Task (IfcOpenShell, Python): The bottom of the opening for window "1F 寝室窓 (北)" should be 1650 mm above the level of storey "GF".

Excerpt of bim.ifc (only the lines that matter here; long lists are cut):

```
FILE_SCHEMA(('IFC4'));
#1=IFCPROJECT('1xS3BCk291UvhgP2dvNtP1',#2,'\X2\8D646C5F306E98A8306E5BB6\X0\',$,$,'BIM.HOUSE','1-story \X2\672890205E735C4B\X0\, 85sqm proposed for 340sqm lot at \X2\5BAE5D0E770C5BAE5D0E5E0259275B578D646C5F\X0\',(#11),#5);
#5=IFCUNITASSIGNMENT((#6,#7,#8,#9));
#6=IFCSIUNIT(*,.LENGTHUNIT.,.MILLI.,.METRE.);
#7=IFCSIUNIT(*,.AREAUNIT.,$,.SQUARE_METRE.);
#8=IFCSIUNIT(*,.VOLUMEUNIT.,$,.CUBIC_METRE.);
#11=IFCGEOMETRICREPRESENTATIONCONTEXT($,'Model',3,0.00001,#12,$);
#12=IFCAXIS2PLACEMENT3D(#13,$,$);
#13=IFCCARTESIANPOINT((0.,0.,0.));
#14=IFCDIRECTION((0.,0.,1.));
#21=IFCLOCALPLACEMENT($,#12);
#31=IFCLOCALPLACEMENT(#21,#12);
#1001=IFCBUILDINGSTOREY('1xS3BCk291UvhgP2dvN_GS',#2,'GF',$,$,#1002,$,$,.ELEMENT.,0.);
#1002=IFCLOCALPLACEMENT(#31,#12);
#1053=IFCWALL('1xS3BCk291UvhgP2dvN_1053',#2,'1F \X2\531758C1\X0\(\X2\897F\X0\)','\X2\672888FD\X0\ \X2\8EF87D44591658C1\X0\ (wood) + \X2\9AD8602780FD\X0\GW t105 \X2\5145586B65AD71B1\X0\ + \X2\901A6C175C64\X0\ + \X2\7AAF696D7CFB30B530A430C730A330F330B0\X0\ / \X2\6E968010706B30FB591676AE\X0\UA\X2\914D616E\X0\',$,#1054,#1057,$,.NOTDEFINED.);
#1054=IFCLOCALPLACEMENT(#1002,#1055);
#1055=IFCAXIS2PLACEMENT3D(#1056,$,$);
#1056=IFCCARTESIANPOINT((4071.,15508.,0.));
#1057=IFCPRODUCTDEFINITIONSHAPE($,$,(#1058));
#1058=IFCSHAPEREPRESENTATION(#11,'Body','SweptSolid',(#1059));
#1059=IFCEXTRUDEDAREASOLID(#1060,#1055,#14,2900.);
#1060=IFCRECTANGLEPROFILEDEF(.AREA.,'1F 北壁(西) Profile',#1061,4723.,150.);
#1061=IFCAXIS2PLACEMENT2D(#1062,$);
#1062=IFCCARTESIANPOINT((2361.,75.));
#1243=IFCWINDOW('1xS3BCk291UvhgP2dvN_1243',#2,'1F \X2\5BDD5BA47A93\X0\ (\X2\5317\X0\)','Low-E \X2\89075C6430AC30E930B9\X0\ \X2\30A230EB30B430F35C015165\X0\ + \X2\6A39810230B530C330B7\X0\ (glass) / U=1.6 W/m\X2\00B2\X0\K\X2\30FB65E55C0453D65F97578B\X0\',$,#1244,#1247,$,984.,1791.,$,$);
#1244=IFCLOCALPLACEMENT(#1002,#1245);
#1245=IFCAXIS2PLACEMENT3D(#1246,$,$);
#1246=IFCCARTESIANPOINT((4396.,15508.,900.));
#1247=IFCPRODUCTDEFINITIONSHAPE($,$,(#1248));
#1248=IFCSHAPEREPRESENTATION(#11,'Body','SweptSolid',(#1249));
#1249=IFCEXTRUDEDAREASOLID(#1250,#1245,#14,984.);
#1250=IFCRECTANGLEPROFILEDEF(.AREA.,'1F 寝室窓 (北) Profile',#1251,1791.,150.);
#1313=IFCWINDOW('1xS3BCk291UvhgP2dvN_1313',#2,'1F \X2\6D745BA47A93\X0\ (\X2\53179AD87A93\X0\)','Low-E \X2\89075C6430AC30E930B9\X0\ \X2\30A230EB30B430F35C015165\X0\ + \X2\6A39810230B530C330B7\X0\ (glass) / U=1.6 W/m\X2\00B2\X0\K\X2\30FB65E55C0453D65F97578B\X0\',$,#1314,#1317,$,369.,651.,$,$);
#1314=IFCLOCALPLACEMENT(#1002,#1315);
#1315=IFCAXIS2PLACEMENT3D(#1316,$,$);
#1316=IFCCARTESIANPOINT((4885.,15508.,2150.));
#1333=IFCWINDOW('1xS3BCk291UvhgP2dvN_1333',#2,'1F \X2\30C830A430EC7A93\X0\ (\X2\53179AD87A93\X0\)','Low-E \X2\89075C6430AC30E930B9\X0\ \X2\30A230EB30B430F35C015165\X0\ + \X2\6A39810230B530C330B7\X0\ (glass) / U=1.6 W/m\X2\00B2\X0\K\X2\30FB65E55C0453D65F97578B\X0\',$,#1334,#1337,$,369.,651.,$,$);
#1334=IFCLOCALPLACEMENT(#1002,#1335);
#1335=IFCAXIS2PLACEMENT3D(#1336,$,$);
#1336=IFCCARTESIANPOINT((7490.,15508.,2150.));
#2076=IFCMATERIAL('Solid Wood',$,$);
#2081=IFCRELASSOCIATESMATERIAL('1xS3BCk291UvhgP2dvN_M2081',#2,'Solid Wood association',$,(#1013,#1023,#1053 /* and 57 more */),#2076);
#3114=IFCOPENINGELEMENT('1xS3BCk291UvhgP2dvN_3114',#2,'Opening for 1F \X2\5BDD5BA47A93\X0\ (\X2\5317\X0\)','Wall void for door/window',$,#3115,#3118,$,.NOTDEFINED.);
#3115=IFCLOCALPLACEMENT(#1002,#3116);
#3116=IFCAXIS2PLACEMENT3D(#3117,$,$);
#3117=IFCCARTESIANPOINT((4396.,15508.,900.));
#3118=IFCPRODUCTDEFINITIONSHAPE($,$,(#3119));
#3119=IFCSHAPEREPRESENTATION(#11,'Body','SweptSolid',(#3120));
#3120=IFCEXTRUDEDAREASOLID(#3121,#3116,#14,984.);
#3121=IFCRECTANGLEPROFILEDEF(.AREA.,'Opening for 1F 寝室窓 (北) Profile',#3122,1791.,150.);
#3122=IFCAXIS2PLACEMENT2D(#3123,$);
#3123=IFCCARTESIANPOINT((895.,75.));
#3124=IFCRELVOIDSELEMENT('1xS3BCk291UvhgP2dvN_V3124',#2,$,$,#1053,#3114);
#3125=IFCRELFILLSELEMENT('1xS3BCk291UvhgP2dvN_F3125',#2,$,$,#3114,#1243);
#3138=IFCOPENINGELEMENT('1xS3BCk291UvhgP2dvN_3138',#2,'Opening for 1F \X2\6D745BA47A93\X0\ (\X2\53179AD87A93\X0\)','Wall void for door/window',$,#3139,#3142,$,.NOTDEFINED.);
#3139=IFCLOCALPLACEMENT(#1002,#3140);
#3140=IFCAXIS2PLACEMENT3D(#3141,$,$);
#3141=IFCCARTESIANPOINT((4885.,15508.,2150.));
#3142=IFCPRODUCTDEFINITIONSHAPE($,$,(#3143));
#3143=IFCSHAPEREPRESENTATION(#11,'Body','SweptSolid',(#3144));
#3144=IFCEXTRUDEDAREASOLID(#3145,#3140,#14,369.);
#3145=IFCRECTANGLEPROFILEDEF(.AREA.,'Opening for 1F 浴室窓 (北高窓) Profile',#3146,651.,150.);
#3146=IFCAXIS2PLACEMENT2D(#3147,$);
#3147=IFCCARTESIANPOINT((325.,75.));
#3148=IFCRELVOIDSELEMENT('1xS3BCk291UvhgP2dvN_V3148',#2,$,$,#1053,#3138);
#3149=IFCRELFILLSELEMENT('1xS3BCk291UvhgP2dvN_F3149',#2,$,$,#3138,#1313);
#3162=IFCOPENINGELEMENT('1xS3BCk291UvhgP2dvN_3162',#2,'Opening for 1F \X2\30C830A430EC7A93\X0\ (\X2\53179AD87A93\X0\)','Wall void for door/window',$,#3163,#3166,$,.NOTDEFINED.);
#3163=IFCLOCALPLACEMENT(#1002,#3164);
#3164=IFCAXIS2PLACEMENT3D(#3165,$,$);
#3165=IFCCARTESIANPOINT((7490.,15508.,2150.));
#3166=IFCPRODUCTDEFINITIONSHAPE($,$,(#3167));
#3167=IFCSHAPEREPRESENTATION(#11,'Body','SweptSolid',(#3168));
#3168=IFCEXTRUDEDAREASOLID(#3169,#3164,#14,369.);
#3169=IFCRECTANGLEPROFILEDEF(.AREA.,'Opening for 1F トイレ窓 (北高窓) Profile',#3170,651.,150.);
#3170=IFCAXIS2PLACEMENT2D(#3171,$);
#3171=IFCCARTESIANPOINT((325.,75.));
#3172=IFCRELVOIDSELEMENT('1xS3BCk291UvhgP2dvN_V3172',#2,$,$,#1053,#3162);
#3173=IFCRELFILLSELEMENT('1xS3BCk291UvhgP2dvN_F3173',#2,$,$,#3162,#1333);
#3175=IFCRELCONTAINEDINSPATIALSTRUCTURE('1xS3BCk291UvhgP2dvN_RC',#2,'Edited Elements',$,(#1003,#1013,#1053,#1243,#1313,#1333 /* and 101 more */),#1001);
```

```python
import numpy as np
import ifcopenshell
import ifcopenshell.api.geometry
import ifcopenshell.geom
import ifcopenshell.util.element
import ifcopenshell.util.placement
import ifcopenshell.util.shape
import ifcopenshell.util.unit

model = ifcopenshell.open("bim.ifc")
unit_scale = ifcopenshell.util.unit.calculate_unit_scale(model)

window = model.by_guid("1xS3BCk291UvhgP2dvN_1243")
opening = window.FillsVoids[0].RelatingOpeningElement
storey = ifcopenshell.util.element.get_container(window, ifc_class="IfcBuildingStorey")
level = ifcopenshell.util.placement.get_local_placement(storey.ObjectPlacement)[2, 3]

# The opening's origin need not be at the sill, so measure its lowest point.
shape = ifcopenshell.geom.create_shape(ifcopenshell.geom.settings(), opening)
bottom = ifcopenshell.util.shape.get_shape_bottom_elevation(shape, shape.geometry) / unit_scale
dz = level + 1.65 / unit_scale - bottom

shift = np.array([0.0, 0.0, dz])
# The window is not placed relative to its opening, so move both.
for product in (opening, window):
    matrix = ifcopenshell.util.placement.get_local_placement(product.ObjectPlacement)
    matrix[:3, 3] += shift
    ifcopenshell.api.geometry.edit_object_placement(model, product=product, matrix=matrix, is_si=False)

print(f"moved by {dz * unit_scale:+.3f} m")

model.write("bim_rev.ifc")
```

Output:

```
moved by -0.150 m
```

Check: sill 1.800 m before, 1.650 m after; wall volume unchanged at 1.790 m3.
